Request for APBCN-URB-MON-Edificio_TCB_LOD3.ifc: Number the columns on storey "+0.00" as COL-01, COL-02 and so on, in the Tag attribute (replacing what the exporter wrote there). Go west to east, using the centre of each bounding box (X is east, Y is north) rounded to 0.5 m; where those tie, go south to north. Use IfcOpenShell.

First a look at what the model holds.

```python
import ifcopenshell
import ifcopenshell.util.element
import ifcopenshell.util.placement

model = ifcopenshell.open("APBCN-URB-MON-Edificio_TCB_LOD3.ifc")
print(model.schema)
storey = next(s for s in model.by_type("IfcBuildingStorey") if s.Name == "+0.00")
columns = [e for e in ifcopenshell.util.element.get_decomposition(storey) if e.is_a("IfcColumn")]
for e in sorted(columns, key=lambda e: e.id()):
    origin = ifcopenshell.util.placement.get_local_placement(e.ObjectPlacement)[:3, 3]
    print(e.id(), e.Tag, e.Name, origin.round(2) + 0.0, sep=" | ")
```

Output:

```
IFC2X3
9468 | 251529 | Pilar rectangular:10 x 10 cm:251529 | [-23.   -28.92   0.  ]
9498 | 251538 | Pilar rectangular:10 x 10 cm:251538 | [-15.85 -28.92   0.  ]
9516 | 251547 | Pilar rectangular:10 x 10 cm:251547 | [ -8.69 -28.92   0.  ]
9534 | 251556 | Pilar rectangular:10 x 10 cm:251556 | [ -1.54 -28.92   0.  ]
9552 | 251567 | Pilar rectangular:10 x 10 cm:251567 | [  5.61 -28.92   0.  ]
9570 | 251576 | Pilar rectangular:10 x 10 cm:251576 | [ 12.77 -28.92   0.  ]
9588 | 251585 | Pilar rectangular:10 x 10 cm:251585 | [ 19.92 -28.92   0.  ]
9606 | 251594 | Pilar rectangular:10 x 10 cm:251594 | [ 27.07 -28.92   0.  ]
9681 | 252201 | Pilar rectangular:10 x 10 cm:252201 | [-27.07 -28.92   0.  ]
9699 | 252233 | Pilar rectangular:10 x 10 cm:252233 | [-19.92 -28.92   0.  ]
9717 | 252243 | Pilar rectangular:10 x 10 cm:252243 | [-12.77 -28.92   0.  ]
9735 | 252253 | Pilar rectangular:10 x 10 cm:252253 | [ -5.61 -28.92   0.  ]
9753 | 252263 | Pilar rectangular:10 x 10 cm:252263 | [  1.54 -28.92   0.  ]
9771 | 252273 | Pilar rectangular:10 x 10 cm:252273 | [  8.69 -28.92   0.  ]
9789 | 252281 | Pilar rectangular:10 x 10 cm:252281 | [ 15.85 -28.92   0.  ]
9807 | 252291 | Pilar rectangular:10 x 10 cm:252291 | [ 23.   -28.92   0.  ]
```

```python
import ifcopenshell
import ifcopenshell.geom
import ifcopenshell.util.element
import ifcopenshell.util.shape

model = ifcopenshell.open("APBCN-URB-MON-Edificio_TCB_LOD3.ifc")
settings = ifcopenshell.geom.settings()
settings.set("use-world-coords", True)


def centre(element):
    shape = ifcopenshell.geom.create_shape(settings, element)
    return ifcopenshell.util.shape.get_bbox_centroid(shape.geometry)


storey = next(s for s in model.by_type("IfcBuildingStorey") if s.Name == "+0.00")
columns = [e for e in ifcopenshell.util.element.get_decomposition(storey) if e.is_a("IfcColumn")]

# Insertion points can sit at a corner or the storey origin, so sort by the geometry (in metres).
centres = {e: centre(e) for e in columns}
columns.sort(key=lambda e: (round(centres[e][0] / 0.5), centres[e][1]))

for i, e in enumerate(columns, start=1):
    number = f"COL-{i:02d}"
    e.Tag = number
    print(e.id(), number)

model.write("APBCN-URB-MON-Edificio_TCB_LOD3_rev.ifc")
```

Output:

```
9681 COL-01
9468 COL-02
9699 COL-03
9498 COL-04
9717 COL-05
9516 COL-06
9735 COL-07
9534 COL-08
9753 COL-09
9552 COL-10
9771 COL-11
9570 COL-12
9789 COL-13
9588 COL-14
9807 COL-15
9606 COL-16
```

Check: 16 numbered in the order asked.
